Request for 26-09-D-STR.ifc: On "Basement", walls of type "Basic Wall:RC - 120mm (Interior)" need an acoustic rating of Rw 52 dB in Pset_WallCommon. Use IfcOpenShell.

First a look at what the model holds.

```python
import ifcopenshell
import ifcopenshell.util.element

model = ifcopenshell.open("26-09-D-STR.ifc")
print(model.schema)
storey = next(s for s in model.by_type("IfcBuildingStorey") if s.Name == "Basement")
walls = [e for e in ifcopenshell.util.element.get_decomposition(storey) if e.is_a("IfcWall")]
seen = {}
for e in walls:
    element_type = ifcopenshell.util.element.get_type(e)
    key = (element_type.Name if element_type != e and element_type else None, ifcopenshell.util.element.get_pset(e, "Pset_WallCommon", "AcousticRating"))
    seen[key] = seen.get(key, 0) + 1
for (name, value), count in sorted(seen.items(), key=str):
    print(count, "x", name, "|", value)
```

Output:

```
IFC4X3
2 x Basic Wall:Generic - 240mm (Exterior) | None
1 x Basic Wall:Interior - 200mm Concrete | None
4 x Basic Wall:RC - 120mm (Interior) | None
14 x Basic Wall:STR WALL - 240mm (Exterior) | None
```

```python
import ifcopenshell
import ifcopenshell.api.pset
import ifcopenshell.util.element

model = ifcopenshell.open("26-09-D-STR.ifc")

storey = next(s for s in model.by_type("IfcBuildingStorey") if s.Name == "Basement")
walls = [e for e in ifcopenshell.util.element.get_decomposition(storey) if e.is_a("IfcWall")]

count = 0
for e in walls:
    element_type = ifcopenshell.util.element.get_type(e)
    if element_type in (None, e) or element_type.Name != "Basic Wall:RC - 120mm (Interior)":
        continue
    # add_pset returns the element's existing set when there is one.
    pset = ifcopenshell.api.pset.add_pset(model, product=e, name="Pset_WallCommon")
    ifcopenshell.api.pset.edit_pset(model, pset=pset, properties={"AcousticRating": "Rw 52 dB"})
    count += 1

print(count, "walls updated")

model.write("26-09-D-STR_edited.ifc")
```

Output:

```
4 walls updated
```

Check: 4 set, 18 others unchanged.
